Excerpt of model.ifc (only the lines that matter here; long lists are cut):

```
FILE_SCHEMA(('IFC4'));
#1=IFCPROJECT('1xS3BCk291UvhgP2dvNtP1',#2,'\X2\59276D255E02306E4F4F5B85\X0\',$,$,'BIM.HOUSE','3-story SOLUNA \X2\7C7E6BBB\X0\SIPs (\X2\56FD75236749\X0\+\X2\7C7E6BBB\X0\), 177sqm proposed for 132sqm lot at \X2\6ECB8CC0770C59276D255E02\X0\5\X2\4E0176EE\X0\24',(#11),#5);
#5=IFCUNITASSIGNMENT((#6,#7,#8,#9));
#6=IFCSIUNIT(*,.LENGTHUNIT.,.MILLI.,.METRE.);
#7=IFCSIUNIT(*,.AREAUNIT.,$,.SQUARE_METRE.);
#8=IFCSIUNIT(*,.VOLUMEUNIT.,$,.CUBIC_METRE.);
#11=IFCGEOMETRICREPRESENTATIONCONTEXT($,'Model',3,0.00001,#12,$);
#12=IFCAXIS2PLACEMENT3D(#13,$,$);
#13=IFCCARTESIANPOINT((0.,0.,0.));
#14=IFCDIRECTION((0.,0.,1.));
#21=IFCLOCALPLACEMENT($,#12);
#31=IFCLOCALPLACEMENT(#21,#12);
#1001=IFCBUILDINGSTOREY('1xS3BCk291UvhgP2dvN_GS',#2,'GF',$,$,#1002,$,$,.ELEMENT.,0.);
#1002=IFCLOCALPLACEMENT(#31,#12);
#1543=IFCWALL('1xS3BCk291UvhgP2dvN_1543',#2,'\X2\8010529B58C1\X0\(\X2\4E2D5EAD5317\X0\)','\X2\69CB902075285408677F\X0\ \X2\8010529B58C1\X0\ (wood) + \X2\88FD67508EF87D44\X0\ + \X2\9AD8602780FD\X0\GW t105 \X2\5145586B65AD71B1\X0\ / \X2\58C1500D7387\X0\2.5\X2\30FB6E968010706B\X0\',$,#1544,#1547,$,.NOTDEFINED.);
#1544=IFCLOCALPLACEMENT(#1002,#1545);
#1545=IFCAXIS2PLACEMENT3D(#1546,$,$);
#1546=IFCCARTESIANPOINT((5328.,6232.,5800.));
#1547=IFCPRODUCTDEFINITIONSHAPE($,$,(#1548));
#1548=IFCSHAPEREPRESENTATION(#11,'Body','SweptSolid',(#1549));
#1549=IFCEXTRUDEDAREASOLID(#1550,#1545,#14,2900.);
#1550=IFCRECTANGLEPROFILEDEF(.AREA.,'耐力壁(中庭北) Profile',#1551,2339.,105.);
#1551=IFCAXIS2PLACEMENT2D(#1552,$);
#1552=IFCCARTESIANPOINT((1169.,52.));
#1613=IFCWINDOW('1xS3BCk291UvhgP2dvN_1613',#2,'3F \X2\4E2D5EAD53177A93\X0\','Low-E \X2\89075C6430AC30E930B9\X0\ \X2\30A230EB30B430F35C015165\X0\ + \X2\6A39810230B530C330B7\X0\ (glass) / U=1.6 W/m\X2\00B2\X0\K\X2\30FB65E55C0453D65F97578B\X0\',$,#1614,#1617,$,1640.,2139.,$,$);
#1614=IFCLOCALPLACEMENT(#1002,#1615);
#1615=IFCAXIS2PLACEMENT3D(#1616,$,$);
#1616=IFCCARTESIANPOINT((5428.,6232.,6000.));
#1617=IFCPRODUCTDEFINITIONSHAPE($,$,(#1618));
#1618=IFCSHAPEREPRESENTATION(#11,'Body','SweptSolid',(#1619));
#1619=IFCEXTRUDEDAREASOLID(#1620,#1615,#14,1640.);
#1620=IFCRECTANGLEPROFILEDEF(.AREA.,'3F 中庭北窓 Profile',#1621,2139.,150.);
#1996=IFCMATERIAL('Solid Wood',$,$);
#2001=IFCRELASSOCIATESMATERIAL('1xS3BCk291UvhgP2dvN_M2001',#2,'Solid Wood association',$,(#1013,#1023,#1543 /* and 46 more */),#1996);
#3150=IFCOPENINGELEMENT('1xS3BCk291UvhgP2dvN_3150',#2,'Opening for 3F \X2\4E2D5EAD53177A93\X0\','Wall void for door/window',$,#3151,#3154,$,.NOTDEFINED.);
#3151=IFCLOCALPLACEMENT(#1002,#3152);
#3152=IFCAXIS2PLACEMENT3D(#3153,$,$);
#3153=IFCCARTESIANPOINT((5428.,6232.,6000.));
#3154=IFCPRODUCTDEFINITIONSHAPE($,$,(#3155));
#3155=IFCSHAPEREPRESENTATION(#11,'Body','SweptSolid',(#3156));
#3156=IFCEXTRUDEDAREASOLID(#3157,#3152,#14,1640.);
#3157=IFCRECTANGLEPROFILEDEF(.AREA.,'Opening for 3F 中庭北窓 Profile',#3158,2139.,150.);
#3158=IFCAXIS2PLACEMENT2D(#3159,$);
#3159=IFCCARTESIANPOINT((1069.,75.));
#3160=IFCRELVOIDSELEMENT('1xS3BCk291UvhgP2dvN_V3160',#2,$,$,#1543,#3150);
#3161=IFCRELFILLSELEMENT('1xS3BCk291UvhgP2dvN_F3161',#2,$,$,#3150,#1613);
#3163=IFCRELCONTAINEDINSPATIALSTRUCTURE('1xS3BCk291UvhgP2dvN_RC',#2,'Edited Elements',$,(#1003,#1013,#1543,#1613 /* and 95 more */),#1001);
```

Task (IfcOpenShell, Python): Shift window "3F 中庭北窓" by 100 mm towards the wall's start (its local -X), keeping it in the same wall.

```python
import ifcopenshell
import ifcopenshell.api.geometry
import ifcopenshell.util.placement
import ifcopenshell.util.unit

model = ifcopenshell.open("model.ifc")
unit_scale = ifcopenshell.util.unit.calculate_unit_scale(model)

window = model.by_guid("1xS3BCk291UvhgP2dvN_1613")
opening = window.FillsVoids[0].RelatingOpeningElement
wall = opening.VoidsElements[0].RelatingBuildingElement

wall_matrix = ifcopenshell.util.placement.get_local_placement(wall.ObjectPlacement)
shift = wall_matrix[:3, 0] * -0.1 / unit_scale
before = ifcopenshell.util.placement.get_local_placement(window.ObjectPlacement)[:3, 3].copy()

# The window is not placed relative to its opening, so move both.
for product in (opening, window):
    matrix = ifcopenshell.util.placement.get_local_placement(product.ObjectPlacement)
    matrix[:3, 3] += shift
    ifcopenshell.api.geometry.edit_object_placement(model, product=product, matrix=matrix, is_si=False)

after = ifcopenshell.util.placement.get_local_placement(window.ObjectPlacement)[:3, 3]
print("window moved by", (after - before).round(3) + 0.0)

model.write("model_rev.ifc")
```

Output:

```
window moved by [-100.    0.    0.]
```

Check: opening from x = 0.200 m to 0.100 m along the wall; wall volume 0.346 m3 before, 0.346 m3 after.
